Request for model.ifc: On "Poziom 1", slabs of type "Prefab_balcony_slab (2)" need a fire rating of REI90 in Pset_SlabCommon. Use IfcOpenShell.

First a look at what the model holds.

```python
import ifcopenshell
import ifcopenshell.util.element

model = ifcopenshell.open("model.ifc")
print(model.schema)
storey = next(s for s in model.by_type("IfcBuildingStorey") if s.Name == "Poziom 1")
slabs = [e for e in ifcopenshell.util.element.get_decomposition(storey) if e.is_a("IfcSlab")]
seen = {}
for e in slabs:
    element_type = ifcopenshell.util.element.get_type(e)
    key = (element_type.Name if element_type != e and element_type else None, ifcopenshell.util.element.get_pset(e, "Pset_SlabCommon", "FireRating"))
    seen[key] = seen.get(key, 0) + 1
for (name, value), count in sorted(seen.items(), key=str):
    print(count, "x", name, "|", value)
```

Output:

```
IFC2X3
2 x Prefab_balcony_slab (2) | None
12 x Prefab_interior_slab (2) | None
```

```python
import ifcopenshell
import ifcopenshell.api.pset
import ifcopenshell.util.element

model = ifcopenshell.open("model.ifc")

storey = next(s for s in model.by_type("IfcBuildingStorey") if s.Name == "Poziom 1")
slabs = [e for e in ifcopenshell.util.element.get_decomposition(storey) if e.is_a("IfcSlab")]

count = 0
for e in slabs:
    element_type = ifcopenshell.util.element.get_type(e)
    if element_type in (None, e) or element_type.Name != "Prefab_balcony_slab (2)":
        continue
    # add_pset returns the element's existing set when there is one.
    pset = ifcopenshell.api.pset.add_pset(model, product=e, name="Pset_SlabCommon")
    ifcopenshell.api.pset.edit_pset(model, pset=pset, properties={"FireRating": "REI90"})
    count += 1

print(count, "slabs updated")

model.write("model_rev.ifc")
```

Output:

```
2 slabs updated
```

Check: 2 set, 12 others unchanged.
